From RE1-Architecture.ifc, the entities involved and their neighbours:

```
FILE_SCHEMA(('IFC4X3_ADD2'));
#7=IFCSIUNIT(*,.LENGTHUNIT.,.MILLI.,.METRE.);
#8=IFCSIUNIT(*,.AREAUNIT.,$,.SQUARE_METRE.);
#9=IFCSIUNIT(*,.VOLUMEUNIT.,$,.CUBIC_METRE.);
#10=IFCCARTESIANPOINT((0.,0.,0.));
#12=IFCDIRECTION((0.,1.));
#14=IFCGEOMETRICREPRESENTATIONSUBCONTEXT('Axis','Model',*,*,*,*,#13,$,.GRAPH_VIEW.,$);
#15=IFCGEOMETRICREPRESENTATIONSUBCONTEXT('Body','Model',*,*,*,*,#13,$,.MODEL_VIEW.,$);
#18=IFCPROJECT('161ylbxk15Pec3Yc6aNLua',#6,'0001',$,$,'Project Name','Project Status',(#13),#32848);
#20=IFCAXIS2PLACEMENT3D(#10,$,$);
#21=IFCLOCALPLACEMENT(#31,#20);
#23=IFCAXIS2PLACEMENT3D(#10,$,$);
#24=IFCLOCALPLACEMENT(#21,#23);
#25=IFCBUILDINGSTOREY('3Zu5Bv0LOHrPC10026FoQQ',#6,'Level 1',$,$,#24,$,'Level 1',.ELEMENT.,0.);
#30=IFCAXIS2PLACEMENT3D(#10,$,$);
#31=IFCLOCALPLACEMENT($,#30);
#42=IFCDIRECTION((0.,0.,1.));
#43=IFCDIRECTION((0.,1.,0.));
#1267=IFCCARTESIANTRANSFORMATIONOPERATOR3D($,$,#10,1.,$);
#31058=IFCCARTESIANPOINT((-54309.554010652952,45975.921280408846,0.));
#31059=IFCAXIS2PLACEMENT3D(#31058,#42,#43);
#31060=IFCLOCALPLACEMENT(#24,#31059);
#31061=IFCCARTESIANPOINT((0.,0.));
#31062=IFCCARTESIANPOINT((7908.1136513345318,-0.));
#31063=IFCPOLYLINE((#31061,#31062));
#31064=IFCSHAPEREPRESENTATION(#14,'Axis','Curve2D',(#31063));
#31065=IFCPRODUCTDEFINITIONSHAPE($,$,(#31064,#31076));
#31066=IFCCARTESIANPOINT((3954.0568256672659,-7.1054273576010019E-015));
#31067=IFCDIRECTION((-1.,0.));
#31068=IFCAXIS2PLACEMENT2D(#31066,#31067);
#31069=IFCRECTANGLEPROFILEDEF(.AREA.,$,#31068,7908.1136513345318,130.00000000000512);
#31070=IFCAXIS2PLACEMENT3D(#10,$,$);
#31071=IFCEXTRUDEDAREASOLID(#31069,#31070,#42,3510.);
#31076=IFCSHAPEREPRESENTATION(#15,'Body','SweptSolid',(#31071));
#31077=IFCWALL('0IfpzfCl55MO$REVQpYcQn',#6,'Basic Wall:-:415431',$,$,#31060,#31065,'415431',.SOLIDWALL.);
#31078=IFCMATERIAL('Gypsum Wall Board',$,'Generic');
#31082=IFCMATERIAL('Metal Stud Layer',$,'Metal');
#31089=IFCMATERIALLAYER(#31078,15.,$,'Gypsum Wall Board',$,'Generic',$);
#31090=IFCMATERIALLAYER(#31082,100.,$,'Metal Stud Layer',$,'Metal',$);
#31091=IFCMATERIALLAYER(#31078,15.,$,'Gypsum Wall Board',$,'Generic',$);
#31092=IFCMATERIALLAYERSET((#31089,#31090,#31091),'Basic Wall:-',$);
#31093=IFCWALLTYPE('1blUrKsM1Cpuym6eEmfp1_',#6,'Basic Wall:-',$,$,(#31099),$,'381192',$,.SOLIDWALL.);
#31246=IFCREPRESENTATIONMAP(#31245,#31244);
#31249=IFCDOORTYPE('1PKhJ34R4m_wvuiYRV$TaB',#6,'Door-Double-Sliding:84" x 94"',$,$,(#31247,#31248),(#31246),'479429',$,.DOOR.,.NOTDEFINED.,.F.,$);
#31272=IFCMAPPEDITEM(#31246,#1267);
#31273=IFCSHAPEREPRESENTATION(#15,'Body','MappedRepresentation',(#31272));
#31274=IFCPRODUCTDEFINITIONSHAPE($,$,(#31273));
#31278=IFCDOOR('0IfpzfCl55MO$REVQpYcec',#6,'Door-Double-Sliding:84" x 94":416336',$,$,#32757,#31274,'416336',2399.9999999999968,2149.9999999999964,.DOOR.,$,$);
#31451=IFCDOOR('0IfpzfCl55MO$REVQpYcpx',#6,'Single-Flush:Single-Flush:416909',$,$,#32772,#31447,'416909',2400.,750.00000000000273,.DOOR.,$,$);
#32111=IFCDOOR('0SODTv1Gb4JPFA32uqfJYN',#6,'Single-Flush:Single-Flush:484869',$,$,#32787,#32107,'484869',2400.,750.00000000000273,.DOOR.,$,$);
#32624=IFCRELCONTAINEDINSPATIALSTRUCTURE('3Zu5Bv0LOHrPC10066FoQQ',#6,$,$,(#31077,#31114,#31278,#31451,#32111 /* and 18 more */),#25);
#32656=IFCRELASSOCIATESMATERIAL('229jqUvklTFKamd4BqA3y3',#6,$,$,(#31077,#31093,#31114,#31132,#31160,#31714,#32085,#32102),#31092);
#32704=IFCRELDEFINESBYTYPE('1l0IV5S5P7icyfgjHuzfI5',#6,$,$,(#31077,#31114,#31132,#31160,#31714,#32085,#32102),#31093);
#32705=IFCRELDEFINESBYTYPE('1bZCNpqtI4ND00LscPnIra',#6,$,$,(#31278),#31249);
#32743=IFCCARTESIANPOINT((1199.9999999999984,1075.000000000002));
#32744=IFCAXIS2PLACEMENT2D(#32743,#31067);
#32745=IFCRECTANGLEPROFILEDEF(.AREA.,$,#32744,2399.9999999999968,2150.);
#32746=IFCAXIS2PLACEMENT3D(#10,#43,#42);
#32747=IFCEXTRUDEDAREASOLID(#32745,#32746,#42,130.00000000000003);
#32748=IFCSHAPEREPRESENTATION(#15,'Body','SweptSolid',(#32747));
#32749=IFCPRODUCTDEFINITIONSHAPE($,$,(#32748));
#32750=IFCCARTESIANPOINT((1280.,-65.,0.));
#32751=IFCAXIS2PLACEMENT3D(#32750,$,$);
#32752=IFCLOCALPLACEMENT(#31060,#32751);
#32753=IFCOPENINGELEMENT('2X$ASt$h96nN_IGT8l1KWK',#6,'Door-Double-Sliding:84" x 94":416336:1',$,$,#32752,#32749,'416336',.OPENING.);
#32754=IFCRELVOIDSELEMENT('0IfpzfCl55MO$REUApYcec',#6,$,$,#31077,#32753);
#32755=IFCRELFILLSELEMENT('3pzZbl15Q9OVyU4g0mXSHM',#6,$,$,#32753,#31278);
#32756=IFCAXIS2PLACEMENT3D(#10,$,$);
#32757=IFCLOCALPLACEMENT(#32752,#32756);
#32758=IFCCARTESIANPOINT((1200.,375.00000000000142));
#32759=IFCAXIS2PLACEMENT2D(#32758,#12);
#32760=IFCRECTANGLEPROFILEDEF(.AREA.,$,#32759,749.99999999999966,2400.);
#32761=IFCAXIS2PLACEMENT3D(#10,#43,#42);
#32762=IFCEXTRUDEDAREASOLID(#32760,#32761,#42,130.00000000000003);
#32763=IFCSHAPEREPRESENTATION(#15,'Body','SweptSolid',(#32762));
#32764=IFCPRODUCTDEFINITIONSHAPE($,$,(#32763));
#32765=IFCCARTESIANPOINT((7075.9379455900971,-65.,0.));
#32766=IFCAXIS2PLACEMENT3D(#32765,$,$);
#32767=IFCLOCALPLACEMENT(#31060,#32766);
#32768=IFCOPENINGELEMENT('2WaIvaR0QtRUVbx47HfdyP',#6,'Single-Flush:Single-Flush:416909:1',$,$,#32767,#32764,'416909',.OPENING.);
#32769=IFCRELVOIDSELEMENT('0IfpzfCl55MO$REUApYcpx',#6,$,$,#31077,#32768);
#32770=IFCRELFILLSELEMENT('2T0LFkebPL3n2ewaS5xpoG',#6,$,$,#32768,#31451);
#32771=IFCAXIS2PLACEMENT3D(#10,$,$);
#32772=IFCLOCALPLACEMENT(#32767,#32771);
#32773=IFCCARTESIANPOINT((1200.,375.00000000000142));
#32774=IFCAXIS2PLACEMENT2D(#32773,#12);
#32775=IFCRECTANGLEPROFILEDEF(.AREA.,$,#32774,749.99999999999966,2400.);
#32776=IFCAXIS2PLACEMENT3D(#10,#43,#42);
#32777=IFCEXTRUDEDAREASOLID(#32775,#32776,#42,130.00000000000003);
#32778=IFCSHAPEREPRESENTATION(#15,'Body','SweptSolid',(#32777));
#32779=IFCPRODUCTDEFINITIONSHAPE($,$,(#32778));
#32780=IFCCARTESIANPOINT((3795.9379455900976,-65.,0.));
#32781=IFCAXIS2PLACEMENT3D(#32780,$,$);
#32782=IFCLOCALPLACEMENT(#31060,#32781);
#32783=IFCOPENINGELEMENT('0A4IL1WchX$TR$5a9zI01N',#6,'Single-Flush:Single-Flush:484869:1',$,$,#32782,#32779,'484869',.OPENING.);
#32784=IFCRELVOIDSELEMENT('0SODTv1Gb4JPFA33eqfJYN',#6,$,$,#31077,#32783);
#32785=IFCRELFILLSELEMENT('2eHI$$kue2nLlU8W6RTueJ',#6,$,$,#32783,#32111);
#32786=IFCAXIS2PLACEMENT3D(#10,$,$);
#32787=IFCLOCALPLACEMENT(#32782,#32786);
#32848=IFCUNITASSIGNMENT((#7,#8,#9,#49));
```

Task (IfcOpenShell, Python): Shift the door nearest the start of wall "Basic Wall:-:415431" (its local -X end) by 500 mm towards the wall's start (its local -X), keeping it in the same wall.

```python
import ifcopenshell
import ifcopenshell.api.geometry
import ifcopenshell.util.placement

model = ifcopenshell.open("RE1-Architecture.ifc")

door = model.by_id(31278)
opening = door.FillsVoids[0].RelatingOpeningElement
wall = opening.VoidsElements[0].RelatingBuildingElement

wall_matrix = ifcopenshell.util.placement.get_local_placement(wall.ObjectPlacement)
shift = wall_matrix[:3, 0] * -500.0
before = ifcopenshell.util.placement.get_local_placement(door.ObjectPlacement)[:3, 3].copy()

# The door is placed relative to its opening, so it follows when the opening moves.
matrix = ifcopenshell.util.placement.get_local_placement(opening.ObjectPlacement)
matrix[:3, 3] += shift
ifcopenshell.api.geometry.edit_object_placement(
    model, product=opening, matrix=matrix, is_si=False, should_transform_children=True
)

after = ifcopenshell.util.placement.get_local_placement(door.ObjectPlacement)[:3, 3]
print("door moved by", (after - before).round(3) + 0.0)

model.write("RE1-Architecture_rev.ifc")
```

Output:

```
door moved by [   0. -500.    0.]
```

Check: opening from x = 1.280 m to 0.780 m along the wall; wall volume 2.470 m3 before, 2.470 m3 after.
